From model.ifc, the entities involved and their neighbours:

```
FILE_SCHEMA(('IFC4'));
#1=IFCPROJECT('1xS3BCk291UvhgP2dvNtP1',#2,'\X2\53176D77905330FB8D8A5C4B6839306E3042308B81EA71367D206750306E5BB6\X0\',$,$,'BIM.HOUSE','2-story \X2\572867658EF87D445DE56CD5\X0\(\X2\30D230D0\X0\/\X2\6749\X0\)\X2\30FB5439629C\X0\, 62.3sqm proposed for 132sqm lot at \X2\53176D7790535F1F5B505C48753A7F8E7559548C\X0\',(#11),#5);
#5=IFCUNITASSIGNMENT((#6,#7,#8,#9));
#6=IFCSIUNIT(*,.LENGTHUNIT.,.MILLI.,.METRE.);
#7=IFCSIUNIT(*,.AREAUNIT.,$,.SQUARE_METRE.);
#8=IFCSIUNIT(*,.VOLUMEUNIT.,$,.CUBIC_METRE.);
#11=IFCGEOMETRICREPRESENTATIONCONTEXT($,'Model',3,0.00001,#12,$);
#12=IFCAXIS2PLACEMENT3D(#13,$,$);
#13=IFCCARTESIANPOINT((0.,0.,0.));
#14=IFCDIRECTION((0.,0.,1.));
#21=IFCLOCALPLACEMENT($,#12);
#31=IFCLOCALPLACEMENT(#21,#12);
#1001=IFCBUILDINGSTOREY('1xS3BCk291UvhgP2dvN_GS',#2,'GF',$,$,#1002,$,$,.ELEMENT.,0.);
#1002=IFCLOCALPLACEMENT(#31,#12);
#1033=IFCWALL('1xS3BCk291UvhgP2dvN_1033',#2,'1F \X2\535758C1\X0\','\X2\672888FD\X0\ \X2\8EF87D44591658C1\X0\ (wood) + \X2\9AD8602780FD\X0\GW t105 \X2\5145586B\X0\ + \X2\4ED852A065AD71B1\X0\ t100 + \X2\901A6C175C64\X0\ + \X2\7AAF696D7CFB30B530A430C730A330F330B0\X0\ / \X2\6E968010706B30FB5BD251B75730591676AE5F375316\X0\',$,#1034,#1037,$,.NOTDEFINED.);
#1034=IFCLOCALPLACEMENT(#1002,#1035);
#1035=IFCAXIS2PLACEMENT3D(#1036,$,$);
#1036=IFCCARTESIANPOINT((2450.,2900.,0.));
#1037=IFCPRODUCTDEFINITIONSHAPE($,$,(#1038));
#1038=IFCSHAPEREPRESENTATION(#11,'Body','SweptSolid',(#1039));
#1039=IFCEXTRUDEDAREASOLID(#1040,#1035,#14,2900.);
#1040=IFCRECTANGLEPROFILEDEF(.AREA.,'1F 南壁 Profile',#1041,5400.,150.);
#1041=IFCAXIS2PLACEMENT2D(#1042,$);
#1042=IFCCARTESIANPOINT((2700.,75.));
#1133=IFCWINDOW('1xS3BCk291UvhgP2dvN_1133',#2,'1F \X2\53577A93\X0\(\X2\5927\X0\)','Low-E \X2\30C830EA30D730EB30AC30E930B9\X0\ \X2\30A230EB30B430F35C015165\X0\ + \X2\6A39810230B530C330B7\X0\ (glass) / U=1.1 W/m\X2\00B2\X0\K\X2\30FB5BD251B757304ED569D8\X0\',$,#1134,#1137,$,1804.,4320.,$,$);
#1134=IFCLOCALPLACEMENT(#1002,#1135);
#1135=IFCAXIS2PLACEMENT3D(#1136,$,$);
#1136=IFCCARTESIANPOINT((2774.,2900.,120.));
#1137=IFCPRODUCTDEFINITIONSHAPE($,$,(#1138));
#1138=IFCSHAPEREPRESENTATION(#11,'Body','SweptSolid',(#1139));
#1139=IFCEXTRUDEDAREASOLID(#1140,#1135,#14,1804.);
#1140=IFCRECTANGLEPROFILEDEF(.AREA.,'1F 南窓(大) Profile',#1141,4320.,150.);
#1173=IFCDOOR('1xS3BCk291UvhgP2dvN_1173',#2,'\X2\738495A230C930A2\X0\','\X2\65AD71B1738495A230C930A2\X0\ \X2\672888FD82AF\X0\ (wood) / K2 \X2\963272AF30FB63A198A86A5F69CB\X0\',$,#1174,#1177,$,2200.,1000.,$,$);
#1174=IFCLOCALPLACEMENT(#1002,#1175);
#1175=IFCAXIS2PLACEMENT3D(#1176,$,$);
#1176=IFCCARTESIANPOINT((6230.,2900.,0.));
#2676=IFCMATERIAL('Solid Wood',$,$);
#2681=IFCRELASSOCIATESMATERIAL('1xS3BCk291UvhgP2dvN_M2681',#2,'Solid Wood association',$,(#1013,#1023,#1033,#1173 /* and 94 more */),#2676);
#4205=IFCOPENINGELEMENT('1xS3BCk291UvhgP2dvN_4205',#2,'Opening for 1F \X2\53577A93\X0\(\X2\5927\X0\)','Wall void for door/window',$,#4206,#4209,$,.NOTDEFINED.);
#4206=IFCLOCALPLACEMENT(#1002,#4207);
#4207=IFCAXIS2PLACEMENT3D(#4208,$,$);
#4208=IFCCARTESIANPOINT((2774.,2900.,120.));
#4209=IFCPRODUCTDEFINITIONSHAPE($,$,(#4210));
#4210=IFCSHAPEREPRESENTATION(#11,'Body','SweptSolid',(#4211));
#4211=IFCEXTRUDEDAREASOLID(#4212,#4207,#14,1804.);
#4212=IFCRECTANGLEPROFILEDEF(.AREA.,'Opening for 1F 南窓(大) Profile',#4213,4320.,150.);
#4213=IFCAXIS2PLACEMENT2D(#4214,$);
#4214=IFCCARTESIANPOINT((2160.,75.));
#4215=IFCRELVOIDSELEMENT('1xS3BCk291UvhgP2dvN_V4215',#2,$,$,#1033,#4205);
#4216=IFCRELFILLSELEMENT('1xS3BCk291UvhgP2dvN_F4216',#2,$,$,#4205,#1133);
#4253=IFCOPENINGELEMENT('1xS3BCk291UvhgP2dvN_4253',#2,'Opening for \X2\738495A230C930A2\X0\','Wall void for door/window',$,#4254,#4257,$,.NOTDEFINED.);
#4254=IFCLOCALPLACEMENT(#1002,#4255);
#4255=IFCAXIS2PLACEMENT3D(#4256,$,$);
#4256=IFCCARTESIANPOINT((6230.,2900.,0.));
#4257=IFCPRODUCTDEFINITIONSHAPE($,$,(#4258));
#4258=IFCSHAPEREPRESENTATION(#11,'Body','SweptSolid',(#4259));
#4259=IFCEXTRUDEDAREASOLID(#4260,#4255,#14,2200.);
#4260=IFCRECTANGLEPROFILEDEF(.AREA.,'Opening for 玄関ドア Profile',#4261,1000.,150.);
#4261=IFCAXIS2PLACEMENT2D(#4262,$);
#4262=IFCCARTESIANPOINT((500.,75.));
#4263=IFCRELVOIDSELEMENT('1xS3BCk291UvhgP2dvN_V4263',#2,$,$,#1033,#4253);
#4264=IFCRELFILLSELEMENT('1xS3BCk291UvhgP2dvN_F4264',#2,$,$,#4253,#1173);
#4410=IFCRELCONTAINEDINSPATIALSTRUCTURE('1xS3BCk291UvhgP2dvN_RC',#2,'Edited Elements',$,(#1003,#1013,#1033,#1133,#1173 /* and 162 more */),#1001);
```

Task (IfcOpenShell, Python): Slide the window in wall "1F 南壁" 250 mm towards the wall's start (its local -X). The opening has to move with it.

```python
import ifcopenshell
import ifcopenshell.api.geometry
import ifcopenshell.util.placement

model = ifcopenshell.open("model.ifc")

window = model.by_guid("1xS3BCk291UvhgP2dvN_1133")
opening = window.FillsVoids[0].RelatingOpeningElement
wall = opening.VoidsElements[0].RelatingBuildingElement

wall_matrix = ifcopenshell.util.placement.get_local_placement(wall.ObjectPlacement)
shift = wall_matrix[:3, 0] * -250.0
before = ifcopenshell.util.placement.get_local_placement(window.ObjectPlacement)[:3, 3].copy()

# The window is not placed relative to its opening, so move both.
for product in (opening, window):
    matrix = ifcopenshell.util.placement.get_local_placement(product.ObjectPlacement)
    matrix[:3, 3] += shift
    ifcopenshell.api.geometry.edit_object_placement(model, product=product, matrix=matrix, is_si=False)

after = ifcopenshell.util.placement.get_local_placement(window.ObjectPlacement)[:3, 3]
print("window moved by", (after - before).round(3) + 0.0)

model.write("model-out.ifc")
```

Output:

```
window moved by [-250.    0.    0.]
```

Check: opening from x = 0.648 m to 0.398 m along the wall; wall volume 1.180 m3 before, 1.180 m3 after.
